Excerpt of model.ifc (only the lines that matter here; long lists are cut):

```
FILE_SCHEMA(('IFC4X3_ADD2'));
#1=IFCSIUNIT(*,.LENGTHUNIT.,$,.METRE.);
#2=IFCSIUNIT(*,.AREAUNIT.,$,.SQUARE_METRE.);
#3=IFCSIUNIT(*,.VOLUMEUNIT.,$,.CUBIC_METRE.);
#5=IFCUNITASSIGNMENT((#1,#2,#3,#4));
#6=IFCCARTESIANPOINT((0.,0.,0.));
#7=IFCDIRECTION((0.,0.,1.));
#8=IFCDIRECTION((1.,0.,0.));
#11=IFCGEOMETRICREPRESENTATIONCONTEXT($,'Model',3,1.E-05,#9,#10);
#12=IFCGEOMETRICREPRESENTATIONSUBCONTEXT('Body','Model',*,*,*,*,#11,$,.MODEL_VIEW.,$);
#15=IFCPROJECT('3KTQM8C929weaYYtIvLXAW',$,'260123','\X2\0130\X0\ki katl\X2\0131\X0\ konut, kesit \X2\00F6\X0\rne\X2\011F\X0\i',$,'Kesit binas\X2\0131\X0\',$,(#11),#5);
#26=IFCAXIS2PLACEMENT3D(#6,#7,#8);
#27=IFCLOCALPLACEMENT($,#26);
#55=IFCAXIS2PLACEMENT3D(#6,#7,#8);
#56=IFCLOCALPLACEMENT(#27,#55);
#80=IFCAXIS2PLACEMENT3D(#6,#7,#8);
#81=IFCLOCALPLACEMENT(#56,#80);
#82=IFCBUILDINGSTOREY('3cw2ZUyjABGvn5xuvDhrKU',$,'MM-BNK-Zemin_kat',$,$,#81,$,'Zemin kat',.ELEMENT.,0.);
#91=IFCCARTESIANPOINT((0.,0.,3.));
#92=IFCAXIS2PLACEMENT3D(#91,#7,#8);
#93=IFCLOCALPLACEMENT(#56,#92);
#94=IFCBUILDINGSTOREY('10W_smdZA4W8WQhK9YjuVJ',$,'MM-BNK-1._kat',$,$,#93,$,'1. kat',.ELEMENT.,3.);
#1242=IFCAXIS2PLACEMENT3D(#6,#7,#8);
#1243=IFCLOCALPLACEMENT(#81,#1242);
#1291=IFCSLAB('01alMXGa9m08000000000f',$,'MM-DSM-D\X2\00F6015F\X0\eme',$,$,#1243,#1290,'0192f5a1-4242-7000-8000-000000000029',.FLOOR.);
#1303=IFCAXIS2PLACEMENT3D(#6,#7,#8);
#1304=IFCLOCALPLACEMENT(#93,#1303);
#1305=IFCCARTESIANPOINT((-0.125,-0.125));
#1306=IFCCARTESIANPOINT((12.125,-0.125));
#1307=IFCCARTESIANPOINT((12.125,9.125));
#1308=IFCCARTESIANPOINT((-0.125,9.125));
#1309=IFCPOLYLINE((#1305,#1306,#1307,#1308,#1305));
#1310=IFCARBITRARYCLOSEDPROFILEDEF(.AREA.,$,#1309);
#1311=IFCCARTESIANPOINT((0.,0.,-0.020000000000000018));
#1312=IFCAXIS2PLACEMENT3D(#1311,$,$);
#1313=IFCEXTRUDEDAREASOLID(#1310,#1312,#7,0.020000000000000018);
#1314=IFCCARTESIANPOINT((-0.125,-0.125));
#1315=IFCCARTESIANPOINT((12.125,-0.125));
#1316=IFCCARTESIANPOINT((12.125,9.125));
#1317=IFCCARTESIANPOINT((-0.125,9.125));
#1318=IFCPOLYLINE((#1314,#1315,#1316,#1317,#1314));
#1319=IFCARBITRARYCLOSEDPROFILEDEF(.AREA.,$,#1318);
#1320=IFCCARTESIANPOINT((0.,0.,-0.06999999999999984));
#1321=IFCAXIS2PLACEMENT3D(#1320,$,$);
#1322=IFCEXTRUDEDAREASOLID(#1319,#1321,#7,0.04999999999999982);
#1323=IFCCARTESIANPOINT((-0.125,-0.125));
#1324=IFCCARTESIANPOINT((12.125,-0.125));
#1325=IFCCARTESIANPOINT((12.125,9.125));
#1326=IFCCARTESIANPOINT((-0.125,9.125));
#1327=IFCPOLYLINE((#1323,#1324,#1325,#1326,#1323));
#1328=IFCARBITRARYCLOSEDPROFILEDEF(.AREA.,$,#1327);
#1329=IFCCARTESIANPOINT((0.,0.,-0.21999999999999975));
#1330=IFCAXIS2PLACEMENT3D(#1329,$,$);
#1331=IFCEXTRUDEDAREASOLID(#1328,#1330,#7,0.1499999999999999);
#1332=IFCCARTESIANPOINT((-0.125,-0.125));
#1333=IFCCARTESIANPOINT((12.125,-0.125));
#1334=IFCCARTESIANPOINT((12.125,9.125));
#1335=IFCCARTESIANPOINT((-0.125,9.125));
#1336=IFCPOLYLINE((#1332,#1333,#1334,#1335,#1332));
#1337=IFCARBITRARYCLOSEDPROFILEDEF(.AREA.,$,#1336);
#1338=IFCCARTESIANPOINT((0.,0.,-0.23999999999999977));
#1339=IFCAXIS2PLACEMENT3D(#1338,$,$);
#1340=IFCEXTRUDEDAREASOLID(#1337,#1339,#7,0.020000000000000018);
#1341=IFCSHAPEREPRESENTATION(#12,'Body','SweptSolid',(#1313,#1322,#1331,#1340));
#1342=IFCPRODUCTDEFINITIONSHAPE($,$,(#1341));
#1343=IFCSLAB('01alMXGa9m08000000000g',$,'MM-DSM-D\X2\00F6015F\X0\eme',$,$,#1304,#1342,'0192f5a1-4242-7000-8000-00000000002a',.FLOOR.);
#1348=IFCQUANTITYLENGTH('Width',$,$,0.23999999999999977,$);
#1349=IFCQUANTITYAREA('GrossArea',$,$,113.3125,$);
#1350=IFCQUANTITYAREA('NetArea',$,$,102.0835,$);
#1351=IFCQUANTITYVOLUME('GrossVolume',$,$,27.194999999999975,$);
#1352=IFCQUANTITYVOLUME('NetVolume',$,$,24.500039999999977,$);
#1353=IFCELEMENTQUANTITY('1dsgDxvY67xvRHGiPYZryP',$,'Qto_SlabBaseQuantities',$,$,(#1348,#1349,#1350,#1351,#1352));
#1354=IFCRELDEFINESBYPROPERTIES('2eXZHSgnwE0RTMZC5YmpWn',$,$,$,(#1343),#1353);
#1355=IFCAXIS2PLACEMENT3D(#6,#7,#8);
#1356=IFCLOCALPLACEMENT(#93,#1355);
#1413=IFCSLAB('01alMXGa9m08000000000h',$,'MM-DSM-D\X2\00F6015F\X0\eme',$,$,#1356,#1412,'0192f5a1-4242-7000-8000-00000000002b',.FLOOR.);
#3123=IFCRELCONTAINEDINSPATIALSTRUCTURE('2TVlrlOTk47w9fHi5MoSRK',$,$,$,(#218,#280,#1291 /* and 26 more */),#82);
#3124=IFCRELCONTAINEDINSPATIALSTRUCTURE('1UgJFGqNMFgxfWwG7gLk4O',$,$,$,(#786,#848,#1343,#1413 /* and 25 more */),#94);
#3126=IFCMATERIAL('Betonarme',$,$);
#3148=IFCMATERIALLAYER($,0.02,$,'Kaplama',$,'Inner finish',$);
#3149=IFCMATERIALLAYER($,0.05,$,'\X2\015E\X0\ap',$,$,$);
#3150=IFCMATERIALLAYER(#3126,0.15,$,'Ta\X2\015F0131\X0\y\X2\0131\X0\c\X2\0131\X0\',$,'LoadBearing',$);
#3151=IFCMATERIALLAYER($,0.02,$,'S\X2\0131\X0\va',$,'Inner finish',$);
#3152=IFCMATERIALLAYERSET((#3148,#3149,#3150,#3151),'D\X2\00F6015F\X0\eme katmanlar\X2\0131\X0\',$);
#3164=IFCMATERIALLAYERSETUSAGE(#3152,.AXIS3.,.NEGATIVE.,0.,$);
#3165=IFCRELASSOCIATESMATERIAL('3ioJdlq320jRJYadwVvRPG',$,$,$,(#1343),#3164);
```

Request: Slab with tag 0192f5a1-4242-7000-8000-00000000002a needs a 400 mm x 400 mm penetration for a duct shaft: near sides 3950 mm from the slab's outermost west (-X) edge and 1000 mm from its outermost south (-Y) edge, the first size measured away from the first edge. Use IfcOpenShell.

```python
import numpy as np
import ifcopenshell
import ifcopenshell.api.feature
import ifcopenshell.api.geometry
import ifcopenshell.api.pset
import ifcopenshell.api.root
import ifcopenshell.geom
import ifcopenshell.util.element
import ifcopenshell.util.placement
import ifcopenshell.util.representation
import ifcopenshell.util.shape
import ifcopenshell.util.unit

model = ifcopenshell.open("model.ifc")
unit_scale = ifcopenshell.util.unit.calculate_unit_scale(model)
area_scale = ifcopenshell.util.unit.calculate_unit_scale(model, "AREAUNIT")
volume_scale = ifcopenshell.util.unit.calculate_unit_scale(model, "VOLUMEUNIT")
settings = ifcopenshell.geom.settings()


def volume(element):
    """Net volume in cubic metres, openings subtracted."""
    shape = ifcopenshell.geom.create_shape(settings, element)
    return ifcopenshell.util.shape.get_volume(shape.geometry)


slab = model.by_id(1343)
before = volume(slab)

# Extent in the slab's own axes, in metres. The edges named are its -X and -Y sides.
slab_shape = ifcopenshell.geom.create_shape(settings, slab)
vertices = ifcopenshell.util.shape.get_vertices(slab_shape.geometry)
x_min, y_min, bottom = vertices.min(axis=0)
top = vertices[:, 2].max()

opening = ifcopenshell.api.root.create_entity(model, ifc_class="IfcOpeningElement", name="Duct shaft opening", predefined_type="OPENING")
context = ifcopenshell.util.representation.get_context(model, "Model", "Body", "MODEL_VIEW")
width, depth = 0.4, 0.4
outline = [(0.0, 0.0), (width, 0.0), (width, depth), (0.0, depth), (0.0, 0.0)]
# Overshoot both faces by 50 mm so the cut is clean.
shape = ifcopenshell.api.geometry.add_slab_representation(
    model, context=context, depth=top - bottom + 0.1, polyline=outline
)
ifcopenshell.api.geometry.assign_representation(model, product=opening, representation=shape)

matrix = ifcopenshell.util.placement.get_local_placement(slab.ObjectPlacement)
matrix[:, 3] = matrix @ np.append(np.array([x_min + 3.95, y_min + 1, bottom - 0.05]) / unit_scale, 1.0)
ifcopenshell.api.geometry.edit_object_placement(model, product=opening, matrix=matrix, is_si=False)
ifcopenshell.api.feature.add_feature(model, feature=opening, element=slab)

after = volume(slab)

# Update the slab's stored quantities.
qto = model.by_id(ifcopenshell.util.element.get_pset(slab, "Qto_SlabBaseQuantities", should_inherit=False)["id"])
ifcopenshell.api.pset.edit_qto(model, qto=qto, properties={
    "NetArea": after / (top - bottom) / area_scale,
    "NetVolume": after / volume_scale,
})

print(f"slab volume {before:.3f} -> {after:.3f} m3")

model.write("model_rev.ifc")
```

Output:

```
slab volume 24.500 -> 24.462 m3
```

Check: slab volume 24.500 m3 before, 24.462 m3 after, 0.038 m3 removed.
